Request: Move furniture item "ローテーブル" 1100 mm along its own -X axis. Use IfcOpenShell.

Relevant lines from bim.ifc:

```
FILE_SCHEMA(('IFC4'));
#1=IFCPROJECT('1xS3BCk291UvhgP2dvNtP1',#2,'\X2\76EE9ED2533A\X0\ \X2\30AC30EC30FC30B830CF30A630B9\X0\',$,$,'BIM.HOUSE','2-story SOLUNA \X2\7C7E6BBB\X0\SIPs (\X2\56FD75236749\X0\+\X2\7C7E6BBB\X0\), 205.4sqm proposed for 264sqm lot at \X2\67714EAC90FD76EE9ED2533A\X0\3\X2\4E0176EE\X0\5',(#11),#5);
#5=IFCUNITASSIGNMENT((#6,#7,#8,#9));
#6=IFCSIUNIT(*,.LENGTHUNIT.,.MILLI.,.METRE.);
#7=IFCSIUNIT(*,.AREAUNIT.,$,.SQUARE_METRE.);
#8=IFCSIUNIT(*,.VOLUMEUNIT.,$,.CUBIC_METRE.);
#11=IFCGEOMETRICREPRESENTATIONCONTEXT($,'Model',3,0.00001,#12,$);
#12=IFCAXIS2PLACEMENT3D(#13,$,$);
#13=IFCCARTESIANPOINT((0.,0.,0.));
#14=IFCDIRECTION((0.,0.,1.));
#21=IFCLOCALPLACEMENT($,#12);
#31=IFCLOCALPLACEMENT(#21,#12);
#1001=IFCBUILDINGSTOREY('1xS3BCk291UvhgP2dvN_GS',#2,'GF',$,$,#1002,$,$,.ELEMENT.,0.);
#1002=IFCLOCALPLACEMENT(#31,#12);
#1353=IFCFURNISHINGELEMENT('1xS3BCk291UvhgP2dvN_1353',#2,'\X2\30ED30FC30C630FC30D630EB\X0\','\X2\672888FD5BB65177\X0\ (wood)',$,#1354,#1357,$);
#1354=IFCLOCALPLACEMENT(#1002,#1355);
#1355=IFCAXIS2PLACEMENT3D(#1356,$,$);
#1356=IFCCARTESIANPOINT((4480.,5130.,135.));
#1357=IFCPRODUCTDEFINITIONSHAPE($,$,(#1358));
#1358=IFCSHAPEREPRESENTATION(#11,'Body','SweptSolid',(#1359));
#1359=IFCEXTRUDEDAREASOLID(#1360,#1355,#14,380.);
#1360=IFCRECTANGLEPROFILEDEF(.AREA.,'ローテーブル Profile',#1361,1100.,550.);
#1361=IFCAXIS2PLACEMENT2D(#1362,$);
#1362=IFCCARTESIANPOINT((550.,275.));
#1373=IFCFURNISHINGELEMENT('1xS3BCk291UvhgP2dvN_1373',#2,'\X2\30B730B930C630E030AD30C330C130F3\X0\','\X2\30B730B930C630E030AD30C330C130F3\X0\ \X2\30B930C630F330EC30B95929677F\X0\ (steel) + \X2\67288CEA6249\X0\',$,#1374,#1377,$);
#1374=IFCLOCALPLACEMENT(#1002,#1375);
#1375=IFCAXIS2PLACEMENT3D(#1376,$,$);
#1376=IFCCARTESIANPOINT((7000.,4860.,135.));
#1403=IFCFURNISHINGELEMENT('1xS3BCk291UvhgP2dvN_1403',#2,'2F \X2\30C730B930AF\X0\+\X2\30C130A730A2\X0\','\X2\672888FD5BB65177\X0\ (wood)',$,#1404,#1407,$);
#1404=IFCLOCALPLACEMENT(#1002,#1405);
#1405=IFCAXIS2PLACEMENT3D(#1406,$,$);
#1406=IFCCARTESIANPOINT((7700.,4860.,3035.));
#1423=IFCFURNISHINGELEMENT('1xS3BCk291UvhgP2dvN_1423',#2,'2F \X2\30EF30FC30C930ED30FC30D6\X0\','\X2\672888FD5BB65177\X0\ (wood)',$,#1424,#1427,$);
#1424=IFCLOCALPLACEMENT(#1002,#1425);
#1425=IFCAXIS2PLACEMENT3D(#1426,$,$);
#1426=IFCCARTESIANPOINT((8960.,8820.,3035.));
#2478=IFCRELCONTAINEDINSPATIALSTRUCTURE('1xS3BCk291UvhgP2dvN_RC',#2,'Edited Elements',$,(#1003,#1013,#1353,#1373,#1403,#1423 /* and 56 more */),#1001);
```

```python
import ifcopenshell
import ifcopenshell.api.geometry
import ifcopenshell.util.placement
import ifcopenshell.util.unit

model = ifcopenshell.open("bim.ifc")
unit_scale = ifcopenshell.util.unit.calculate_unit_scale(model)

item = model.by_id(1353)
matrix = ifcopenshell.util.placement.get_local_placement(item.ObjectPlacement)
matrix[:3, 3] -= matrix[:3, 0] * 1.1 / unit_scale
ifcopenshell.api.geometry.edit_object_placement(model, product=item, matrix=matrix, is_si=False)

print(ifcopenshell.util.placement.get_local_placement(item.ObjectPlacement).round(3) + 0.0)

model.write("bim_updated.ifc")
```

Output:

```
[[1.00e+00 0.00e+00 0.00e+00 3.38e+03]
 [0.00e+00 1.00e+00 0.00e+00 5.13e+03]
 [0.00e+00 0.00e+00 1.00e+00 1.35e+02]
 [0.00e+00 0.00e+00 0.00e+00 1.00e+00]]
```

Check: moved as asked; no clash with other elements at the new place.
